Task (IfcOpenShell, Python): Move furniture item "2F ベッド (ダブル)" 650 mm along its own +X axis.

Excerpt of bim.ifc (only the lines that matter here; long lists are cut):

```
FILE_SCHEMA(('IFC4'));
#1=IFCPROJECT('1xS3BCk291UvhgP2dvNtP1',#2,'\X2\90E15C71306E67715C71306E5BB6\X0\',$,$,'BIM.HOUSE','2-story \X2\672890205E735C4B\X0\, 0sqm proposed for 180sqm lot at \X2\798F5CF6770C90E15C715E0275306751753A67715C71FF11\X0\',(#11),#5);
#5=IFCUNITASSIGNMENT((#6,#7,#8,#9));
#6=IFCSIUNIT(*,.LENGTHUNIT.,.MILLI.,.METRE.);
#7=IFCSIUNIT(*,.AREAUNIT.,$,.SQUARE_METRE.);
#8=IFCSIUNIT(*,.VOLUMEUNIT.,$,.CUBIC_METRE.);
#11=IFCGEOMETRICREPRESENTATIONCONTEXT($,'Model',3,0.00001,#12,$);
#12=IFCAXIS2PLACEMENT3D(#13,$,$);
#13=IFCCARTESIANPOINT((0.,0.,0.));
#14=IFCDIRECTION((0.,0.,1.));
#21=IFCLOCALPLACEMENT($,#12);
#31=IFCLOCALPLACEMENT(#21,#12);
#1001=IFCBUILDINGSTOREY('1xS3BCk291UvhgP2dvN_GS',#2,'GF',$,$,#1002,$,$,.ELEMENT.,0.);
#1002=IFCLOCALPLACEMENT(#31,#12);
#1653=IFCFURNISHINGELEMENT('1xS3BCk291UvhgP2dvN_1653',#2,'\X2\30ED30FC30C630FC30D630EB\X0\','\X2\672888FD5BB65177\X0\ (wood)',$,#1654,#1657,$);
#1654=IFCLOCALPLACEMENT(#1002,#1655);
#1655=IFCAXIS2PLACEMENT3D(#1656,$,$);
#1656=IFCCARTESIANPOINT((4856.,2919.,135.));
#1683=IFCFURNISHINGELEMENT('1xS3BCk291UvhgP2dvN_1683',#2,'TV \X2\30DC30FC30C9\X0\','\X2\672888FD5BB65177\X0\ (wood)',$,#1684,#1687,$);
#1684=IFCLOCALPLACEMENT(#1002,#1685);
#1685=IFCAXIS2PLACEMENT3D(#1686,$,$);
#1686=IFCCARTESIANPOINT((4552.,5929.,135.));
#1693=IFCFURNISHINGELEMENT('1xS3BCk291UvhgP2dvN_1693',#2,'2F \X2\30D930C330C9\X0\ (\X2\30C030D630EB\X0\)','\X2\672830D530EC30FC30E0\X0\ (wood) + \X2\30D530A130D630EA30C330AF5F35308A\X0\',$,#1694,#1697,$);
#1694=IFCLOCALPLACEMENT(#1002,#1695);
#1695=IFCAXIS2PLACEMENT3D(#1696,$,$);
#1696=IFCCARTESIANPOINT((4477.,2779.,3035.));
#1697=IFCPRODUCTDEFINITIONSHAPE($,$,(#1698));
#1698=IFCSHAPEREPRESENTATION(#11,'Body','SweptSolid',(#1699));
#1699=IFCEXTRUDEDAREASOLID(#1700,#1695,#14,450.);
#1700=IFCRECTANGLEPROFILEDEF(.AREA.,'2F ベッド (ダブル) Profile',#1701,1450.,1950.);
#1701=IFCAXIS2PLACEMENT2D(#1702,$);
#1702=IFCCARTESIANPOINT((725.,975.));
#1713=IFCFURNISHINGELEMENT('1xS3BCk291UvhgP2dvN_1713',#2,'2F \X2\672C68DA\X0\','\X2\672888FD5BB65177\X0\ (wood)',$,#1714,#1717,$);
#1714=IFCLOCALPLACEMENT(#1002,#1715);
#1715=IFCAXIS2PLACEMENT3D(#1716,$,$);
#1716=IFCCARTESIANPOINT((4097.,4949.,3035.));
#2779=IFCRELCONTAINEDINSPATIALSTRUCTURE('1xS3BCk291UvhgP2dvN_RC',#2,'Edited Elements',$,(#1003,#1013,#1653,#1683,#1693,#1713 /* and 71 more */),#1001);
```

```python
import ifcopenshell
import ifcopenshell.api.geometry
import ifcopenshell.util.placement

model = ifcopenshell.open("bim.ifc")

item = model.by_guid("1xS3BCk291UvhgP2dvN_1693")
matrix = ifcopenshell.util.placement.get_local_placement(item.ObjectPlacement)
matrix[:3, 3] += matrix[:3, 0] * 650.0
ifcopenshell.api.geometry.edit_object_placement(model, product=item, matrix=matrix, is_si=False)

print(ifcopenshell.util.placement.get_local_placement(item.ObjectPlacement).round(3) + 0.0)

model.write("bim_edited.ifc")
```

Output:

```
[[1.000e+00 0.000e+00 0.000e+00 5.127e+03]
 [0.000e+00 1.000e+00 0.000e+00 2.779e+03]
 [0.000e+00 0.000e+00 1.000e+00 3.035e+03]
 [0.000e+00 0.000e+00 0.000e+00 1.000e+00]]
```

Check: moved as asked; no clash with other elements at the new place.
